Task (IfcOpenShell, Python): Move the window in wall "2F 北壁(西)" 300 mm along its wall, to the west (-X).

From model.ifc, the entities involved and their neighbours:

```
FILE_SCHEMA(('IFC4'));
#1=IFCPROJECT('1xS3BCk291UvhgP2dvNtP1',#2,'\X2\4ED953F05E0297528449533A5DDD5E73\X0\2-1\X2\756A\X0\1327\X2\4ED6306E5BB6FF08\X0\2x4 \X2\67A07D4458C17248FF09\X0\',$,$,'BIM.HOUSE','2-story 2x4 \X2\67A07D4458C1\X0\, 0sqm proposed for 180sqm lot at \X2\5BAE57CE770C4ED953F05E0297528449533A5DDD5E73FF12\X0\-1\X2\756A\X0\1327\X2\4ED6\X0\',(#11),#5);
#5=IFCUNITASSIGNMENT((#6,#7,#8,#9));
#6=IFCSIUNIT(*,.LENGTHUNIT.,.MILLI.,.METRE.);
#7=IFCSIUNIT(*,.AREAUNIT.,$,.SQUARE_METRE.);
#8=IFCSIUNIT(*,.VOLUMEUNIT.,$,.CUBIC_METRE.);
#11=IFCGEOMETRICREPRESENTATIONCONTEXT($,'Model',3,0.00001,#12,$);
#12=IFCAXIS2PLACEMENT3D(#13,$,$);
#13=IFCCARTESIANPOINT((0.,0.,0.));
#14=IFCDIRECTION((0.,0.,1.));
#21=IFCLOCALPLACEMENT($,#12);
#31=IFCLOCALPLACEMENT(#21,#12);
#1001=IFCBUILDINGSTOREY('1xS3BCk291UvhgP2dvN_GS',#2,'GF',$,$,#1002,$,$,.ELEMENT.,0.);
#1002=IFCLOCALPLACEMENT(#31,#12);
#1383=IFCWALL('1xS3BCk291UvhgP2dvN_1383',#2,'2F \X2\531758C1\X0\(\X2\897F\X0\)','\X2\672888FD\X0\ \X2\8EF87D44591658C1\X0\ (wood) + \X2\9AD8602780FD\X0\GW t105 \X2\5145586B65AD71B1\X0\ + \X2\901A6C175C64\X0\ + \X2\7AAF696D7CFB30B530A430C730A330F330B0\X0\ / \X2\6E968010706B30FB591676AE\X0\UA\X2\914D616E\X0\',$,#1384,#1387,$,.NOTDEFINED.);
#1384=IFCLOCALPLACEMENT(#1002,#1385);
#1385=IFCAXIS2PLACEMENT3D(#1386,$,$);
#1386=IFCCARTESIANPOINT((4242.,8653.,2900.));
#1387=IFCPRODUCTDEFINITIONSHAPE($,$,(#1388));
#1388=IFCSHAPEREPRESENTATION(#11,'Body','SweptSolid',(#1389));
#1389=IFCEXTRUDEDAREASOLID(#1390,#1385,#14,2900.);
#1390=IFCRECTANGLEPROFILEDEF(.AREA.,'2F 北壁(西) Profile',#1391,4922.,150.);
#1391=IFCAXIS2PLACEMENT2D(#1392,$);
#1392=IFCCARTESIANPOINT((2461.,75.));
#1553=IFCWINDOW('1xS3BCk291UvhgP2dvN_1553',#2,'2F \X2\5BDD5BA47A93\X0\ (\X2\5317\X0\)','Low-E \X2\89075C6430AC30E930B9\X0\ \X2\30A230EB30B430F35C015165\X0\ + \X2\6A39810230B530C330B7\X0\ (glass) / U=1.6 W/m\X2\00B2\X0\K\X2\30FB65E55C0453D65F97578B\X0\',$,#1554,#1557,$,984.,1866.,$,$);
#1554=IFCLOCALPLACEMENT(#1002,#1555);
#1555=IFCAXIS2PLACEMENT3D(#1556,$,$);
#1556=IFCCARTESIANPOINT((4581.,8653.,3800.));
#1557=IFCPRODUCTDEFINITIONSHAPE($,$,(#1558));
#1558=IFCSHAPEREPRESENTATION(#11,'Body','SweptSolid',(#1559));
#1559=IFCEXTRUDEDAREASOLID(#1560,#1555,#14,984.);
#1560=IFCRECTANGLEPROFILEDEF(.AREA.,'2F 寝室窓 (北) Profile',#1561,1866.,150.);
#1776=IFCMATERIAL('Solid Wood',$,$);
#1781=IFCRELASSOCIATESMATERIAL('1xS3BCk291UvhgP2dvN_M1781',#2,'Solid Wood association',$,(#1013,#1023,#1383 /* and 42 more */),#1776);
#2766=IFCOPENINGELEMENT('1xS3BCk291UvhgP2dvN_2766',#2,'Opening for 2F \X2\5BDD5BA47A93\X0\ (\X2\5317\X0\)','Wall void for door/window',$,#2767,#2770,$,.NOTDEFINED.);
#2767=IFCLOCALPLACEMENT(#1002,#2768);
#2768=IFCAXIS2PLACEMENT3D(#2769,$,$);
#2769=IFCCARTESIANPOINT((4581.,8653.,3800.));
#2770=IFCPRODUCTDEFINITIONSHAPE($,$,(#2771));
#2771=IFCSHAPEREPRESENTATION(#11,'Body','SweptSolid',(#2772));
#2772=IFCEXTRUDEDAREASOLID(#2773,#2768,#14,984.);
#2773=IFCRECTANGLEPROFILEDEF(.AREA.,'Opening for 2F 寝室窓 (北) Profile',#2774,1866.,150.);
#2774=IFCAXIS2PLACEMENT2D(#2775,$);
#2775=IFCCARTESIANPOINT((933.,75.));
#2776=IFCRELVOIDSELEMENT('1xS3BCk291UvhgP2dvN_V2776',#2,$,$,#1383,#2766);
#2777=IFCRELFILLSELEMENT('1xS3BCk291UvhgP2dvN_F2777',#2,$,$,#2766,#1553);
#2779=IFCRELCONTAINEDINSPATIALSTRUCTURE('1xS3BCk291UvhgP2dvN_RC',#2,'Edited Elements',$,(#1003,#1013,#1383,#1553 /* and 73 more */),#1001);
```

```python
import ifcopenshell
import ifcopenshell.api.geometry
import ifcopenshell.util.placement

model = ifcopenshell.open("model.ifc")

window = model.by_id(1553)
opening = window.FillsVoids[0].RelatingOpeningElement
wall = opening.VoidsElements[0].RelatingBuildingElement

wall_matrix = ifcopenshell.util.placement.get_local_placement(wall.ObjectPlacement)
shift = wall_matrix[:3, 0] * -300.0
before = ifcopenshell.util.placement.get_local_placement(window.ObjectPlacement)[:3, 3].copy()

# The window is not placed relative to its opening, so move both.
for product in (opening, window):
    matrix = ifcopenshell.util.placement.get_local_placement(product.ObjectPlacement)
    matrix[:3, 3] += shift
    ifcopenshell.api.geometry.edit_object_placement(model, product=product, matrix=matrix, is_si=False)

after = ifcopenshell.util.placement.get_local_placement(window.ObjectPlacement)[:3, 3]
print("window moved by", (after - before).round(3) + 0.0)

model.write("model_rev.ifc")
```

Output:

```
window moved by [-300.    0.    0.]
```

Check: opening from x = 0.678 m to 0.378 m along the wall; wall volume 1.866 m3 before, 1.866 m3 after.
